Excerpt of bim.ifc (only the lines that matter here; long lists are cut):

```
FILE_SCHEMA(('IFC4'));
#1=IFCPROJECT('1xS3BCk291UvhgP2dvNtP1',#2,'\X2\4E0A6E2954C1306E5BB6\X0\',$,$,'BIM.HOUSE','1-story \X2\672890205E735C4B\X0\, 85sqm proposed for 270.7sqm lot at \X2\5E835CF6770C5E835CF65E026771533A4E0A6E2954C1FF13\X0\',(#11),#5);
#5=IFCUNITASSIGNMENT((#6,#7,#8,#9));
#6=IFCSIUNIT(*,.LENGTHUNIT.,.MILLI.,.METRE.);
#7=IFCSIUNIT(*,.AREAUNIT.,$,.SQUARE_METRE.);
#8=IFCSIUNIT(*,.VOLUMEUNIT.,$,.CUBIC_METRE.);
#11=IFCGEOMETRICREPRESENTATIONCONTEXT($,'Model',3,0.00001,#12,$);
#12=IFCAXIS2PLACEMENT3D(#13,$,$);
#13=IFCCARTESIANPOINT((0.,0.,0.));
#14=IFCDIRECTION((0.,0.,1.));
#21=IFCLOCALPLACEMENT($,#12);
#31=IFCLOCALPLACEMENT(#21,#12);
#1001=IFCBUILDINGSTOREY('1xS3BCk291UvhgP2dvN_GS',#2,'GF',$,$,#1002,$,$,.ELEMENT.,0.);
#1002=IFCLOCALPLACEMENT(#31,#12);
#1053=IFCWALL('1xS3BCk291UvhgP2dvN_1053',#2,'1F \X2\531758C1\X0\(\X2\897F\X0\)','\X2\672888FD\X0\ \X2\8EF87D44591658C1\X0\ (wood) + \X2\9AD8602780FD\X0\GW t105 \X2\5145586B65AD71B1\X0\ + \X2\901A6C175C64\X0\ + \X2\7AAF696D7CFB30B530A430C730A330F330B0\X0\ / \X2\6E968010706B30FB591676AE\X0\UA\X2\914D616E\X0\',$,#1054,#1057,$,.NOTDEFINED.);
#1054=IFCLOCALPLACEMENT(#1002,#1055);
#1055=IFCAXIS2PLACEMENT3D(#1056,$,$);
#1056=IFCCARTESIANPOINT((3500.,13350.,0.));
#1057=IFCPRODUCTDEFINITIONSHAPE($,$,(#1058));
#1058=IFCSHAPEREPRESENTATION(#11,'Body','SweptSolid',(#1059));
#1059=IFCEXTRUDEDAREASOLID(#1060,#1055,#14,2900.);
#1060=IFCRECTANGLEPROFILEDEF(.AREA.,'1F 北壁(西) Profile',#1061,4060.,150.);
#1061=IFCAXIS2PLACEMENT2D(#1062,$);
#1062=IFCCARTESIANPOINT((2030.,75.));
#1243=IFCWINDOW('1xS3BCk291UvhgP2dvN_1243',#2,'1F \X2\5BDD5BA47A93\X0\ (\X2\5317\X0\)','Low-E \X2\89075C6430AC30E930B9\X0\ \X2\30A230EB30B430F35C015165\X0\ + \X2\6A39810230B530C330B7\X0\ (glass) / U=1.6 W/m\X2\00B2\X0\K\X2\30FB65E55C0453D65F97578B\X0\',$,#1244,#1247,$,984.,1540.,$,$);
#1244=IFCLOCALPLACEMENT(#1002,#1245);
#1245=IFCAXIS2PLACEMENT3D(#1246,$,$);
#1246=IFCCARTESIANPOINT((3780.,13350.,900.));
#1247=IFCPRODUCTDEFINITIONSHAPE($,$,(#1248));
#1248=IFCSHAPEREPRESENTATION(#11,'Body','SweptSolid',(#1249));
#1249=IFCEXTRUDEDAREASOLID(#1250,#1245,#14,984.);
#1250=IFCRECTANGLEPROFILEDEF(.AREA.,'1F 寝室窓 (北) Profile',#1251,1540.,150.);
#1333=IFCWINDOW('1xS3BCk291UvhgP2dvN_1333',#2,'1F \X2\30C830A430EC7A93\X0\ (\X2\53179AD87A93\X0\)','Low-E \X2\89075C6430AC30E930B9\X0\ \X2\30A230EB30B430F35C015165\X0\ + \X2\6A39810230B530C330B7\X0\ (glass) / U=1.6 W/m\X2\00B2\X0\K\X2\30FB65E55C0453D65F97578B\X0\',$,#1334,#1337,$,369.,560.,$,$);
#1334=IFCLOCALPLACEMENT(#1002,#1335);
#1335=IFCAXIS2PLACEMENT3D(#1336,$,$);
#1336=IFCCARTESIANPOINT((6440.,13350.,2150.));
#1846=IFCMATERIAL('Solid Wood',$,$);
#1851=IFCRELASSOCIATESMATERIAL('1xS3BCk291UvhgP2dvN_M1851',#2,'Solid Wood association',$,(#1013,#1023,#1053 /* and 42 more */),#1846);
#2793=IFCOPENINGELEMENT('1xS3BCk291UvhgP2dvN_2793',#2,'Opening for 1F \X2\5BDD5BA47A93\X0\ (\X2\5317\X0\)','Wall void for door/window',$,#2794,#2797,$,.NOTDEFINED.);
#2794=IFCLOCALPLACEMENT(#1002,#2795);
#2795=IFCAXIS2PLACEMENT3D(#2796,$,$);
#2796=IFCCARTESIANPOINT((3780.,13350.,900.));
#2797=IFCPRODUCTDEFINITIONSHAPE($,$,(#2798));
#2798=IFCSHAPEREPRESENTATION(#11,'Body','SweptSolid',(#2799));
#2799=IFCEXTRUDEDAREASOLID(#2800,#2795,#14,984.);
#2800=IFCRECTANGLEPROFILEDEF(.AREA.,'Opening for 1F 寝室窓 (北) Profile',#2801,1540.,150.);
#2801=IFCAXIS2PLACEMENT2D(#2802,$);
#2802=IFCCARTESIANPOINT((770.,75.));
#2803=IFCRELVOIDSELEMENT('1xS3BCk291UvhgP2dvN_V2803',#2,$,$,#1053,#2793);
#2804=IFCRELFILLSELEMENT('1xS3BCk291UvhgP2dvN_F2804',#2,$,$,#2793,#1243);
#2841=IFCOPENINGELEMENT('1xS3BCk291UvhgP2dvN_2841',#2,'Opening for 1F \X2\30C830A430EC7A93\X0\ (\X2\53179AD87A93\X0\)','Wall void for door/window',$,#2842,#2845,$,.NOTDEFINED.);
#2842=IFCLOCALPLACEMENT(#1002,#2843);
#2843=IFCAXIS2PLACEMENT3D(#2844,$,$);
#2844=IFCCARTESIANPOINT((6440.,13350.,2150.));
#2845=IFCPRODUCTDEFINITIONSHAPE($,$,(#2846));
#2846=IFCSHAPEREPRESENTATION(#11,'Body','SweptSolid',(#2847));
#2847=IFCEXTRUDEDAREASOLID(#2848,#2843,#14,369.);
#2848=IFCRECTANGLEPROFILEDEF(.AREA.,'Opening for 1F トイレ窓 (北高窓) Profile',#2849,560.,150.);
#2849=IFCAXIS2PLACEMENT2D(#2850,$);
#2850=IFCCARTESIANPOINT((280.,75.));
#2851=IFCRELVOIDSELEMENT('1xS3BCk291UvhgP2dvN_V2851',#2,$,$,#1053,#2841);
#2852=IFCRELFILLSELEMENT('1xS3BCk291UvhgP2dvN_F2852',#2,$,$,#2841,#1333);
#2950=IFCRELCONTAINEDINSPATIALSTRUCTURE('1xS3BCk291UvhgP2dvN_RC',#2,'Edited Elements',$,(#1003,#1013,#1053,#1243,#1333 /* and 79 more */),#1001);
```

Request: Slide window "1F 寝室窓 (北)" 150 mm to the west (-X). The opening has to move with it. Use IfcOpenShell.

```python
import ifcopenshell
import ifcopenshell.api.geometry
import ifcopenshell.util.placement
import ifcopenshell.util.unit

model = ifcopenshell.open("bim.ifc")
unit_scale = ifcopenshell.util.unit.calculate_unit_scale(model)

window = model.by_id(1243)
opening = window.FillsVoids[0].RelatingOpeningElement
wall = opening.VoidsElements[0].RelatingBuildingElement

wall_matrix = ifcopenshell.util.placement.get_local_placement(wall.ObjectPlacement)
shift = wall_matrix[:3, 0] * -0.15 / unit_scale
before = ifcopenshell.util.placement.get_local_placement(window.ObjectPlacement)[:3, 3].copy()

# The window is not placed relative to its opening, so move both.
for product in (opening, window):
    matrix = ifcopenshell.util.placement.get_local_placement(product.ObjectPlacement)
    matrix[:3, 3] += shift
    ifcopenshell.api.geometry.edit_object_placement(model, product=product, matrix=matrix, is_si=False)

after = ifcopenshell.util.placement.get_local_placement(window.ObjectPlacement)[:3, 3]
print("window moved by", (after - before).round(3) + 0.0)

model.write("bim_rev.ifc")
```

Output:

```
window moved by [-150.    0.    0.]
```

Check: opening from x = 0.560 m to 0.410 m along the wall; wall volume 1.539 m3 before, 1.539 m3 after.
